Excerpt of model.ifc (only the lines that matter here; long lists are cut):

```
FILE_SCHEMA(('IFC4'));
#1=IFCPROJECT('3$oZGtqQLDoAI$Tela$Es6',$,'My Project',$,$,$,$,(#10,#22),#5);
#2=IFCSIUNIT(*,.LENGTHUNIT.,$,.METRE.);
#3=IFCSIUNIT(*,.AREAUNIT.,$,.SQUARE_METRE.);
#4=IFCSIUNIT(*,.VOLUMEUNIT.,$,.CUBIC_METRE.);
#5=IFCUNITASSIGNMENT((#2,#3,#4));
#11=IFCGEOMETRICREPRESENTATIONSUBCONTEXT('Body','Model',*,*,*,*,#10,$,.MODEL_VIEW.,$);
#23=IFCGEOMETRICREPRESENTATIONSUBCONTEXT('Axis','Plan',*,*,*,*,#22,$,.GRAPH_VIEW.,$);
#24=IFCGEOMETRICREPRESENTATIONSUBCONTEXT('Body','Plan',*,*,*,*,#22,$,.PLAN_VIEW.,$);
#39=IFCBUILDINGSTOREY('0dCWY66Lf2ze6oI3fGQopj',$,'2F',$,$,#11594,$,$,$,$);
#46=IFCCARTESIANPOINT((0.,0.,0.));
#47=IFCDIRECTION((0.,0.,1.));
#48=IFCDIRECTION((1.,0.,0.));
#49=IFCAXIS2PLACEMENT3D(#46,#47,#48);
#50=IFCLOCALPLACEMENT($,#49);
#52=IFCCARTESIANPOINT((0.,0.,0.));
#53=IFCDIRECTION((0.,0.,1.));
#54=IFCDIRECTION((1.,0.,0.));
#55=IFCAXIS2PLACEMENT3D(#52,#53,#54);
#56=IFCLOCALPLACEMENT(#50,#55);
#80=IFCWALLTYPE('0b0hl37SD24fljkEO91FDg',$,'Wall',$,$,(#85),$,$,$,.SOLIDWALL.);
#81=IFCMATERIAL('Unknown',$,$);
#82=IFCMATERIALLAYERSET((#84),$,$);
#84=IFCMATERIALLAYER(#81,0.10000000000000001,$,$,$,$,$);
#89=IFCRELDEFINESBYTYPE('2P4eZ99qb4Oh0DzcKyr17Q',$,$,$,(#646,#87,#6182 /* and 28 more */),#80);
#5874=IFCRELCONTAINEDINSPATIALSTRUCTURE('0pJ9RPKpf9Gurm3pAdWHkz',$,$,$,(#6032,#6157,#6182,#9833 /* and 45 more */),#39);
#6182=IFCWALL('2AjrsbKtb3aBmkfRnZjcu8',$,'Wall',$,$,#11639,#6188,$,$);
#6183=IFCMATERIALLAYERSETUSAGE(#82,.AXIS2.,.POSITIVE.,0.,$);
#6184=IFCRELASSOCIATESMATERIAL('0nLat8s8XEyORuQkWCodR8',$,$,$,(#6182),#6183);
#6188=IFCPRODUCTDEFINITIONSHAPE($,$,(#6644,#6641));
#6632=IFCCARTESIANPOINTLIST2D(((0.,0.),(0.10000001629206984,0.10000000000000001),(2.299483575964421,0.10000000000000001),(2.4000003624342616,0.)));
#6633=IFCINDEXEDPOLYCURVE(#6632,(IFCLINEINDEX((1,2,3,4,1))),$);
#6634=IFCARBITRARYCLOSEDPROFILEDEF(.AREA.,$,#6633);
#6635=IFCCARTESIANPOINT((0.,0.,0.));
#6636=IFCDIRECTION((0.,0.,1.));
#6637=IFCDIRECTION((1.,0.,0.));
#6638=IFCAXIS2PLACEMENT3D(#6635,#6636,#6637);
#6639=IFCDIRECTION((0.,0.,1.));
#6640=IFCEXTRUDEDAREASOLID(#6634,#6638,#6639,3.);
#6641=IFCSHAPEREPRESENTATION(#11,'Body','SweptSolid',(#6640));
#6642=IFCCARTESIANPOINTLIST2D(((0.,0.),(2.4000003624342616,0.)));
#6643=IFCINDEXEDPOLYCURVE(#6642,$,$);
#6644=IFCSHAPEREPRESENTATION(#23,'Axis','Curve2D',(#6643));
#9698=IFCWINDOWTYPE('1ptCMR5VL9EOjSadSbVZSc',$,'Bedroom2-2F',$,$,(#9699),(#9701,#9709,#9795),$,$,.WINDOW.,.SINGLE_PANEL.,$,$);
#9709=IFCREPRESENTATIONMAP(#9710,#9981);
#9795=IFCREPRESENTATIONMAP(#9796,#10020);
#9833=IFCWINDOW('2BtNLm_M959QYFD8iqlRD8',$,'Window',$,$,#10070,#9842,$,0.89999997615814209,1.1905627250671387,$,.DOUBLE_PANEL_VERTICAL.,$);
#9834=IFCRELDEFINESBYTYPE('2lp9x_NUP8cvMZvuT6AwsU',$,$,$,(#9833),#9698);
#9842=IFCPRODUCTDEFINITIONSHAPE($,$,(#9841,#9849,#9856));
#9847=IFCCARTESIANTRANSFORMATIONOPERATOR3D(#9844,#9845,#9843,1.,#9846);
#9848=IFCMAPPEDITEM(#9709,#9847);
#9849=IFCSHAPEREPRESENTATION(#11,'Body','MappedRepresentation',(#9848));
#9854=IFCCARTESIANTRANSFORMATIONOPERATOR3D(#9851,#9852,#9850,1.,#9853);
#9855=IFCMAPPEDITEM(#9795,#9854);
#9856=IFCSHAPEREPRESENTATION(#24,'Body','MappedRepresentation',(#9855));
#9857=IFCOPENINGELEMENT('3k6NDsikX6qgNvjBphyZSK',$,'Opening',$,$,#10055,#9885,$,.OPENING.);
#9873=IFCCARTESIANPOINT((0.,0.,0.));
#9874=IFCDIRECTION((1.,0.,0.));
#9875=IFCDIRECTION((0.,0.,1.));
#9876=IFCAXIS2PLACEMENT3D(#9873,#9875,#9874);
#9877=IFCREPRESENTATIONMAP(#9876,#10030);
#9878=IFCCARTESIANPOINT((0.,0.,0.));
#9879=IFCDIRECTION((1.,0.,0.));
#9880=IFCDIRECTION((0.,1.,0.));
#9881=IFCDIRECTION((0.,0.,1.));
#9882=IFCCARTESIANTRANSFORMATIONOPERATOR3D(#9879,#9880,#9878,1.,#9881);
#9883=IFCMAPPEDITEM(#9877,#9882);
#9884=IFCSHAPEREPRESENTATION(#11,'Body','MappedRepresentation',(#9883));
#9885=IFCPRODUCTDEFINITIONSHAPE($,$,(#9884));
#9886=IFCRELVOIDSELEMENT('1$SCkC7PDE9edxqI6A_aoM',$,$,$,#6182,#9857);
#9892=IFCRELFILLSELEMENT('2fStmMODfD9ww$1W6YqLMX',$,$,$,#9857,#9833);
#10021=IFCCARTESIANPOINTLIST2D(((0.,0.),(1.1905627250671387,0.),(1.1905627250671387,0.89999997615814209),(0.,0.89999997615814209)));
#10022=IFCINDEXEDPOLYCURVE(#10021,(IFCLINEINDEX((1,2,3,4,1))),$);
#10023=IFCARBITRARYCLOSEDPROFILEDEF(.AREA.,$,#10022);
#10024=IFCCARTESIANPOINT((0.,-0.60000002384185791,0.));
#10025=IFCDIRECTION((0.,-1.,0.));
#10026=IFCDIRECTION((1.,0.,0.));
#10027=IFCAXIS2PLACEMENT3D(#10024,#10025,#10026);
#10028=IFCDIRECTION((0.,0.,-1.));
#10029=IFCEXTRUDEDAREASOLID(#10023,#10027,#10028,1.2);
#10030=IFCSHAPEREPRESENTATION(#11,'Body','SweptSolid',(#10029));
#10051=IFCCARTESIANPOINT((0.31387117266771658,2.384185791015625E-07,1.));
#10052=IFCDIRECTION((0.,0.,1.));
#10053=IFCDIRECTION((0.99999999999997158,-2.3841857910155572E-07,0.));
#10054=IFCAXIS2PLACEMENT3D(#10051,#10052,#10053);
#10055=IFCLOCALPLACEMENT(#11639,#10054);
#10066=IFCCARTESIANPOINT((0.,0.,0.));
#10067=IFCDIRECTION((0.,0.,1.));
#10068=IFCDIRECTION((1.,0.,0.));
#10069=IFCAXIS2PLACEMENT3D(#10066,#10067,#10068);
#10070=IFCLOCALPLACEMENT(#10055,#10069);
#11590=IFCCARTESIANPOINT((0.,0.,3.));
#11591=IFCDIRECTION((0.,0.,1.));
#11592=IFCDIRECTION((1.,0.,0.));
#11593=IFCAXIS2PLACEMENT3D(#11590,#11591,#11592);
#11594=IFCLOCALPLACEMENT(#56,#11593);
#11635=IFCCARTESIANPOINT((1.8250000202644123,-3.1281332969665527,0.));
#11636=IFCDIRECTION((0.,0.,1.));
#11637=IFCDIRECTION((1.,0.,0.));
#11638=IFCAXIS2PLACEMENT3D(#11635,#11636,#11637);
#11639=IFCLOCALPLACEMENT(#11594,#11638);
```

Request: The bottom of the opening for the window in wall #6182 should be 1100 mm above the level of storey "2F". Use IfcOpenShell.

```python
import numpy as np
import ifcopenshell
import ifcopenshell.api.geometry
import ifcopenshell.geom
import ifcopenshell.util.element
import ifcopenshell.util.placement
import ifcopenshell.util.shape
import ifcopenshell.util.unit

model = ifcopenshell.open("model.ifc")
unit_scale = ifcopenshell.util.unit.calculate_unit_scale(model)

window = model.by_guid("2BtNLm_M959QYFD8iqlRD8")
opening = window.FillsVoids[0].RelatingOpeningElement
storey = ifcopenshell.util.element.get_container(window, ifc_class="IfcBuildingStorey")
level = ifcopenshell.util.placement.get_local_placement(storey.ObjectPlacement)[2, 3]

# The opening's origin need not be at the sill, so measure its lowest point.
shape = ifcopenshell.geom.create_shape(ifcopenshell.geom.settings(), opening)
bottom = ifcopenshell.util.shape.get_shape_bottom_elevation(shape, shape.geometry) / unit_scale
dz = level + 1.1 / unit_scale - bottom

shift = np.array([0.0, 0.0, dz])
# The window is placed relative to its opening, so it follows when the opening moves.
matrix = ifcopenshell.util.placement.get_local_placement(opening.ObjectPlacement)
matrix[:3, 3] += shift
ifcopenshell.api.geometry.edit_object_placement(
    model, product=opening, matrix=matrix, is_si=False, should_transform_children=True
)

print(f"moved by {dz * unit_scale:+.3f} m")

model.write("model_v2.ifc")
```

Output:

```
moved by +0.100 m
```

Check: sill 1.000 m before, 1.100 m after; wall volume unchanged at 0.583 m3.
